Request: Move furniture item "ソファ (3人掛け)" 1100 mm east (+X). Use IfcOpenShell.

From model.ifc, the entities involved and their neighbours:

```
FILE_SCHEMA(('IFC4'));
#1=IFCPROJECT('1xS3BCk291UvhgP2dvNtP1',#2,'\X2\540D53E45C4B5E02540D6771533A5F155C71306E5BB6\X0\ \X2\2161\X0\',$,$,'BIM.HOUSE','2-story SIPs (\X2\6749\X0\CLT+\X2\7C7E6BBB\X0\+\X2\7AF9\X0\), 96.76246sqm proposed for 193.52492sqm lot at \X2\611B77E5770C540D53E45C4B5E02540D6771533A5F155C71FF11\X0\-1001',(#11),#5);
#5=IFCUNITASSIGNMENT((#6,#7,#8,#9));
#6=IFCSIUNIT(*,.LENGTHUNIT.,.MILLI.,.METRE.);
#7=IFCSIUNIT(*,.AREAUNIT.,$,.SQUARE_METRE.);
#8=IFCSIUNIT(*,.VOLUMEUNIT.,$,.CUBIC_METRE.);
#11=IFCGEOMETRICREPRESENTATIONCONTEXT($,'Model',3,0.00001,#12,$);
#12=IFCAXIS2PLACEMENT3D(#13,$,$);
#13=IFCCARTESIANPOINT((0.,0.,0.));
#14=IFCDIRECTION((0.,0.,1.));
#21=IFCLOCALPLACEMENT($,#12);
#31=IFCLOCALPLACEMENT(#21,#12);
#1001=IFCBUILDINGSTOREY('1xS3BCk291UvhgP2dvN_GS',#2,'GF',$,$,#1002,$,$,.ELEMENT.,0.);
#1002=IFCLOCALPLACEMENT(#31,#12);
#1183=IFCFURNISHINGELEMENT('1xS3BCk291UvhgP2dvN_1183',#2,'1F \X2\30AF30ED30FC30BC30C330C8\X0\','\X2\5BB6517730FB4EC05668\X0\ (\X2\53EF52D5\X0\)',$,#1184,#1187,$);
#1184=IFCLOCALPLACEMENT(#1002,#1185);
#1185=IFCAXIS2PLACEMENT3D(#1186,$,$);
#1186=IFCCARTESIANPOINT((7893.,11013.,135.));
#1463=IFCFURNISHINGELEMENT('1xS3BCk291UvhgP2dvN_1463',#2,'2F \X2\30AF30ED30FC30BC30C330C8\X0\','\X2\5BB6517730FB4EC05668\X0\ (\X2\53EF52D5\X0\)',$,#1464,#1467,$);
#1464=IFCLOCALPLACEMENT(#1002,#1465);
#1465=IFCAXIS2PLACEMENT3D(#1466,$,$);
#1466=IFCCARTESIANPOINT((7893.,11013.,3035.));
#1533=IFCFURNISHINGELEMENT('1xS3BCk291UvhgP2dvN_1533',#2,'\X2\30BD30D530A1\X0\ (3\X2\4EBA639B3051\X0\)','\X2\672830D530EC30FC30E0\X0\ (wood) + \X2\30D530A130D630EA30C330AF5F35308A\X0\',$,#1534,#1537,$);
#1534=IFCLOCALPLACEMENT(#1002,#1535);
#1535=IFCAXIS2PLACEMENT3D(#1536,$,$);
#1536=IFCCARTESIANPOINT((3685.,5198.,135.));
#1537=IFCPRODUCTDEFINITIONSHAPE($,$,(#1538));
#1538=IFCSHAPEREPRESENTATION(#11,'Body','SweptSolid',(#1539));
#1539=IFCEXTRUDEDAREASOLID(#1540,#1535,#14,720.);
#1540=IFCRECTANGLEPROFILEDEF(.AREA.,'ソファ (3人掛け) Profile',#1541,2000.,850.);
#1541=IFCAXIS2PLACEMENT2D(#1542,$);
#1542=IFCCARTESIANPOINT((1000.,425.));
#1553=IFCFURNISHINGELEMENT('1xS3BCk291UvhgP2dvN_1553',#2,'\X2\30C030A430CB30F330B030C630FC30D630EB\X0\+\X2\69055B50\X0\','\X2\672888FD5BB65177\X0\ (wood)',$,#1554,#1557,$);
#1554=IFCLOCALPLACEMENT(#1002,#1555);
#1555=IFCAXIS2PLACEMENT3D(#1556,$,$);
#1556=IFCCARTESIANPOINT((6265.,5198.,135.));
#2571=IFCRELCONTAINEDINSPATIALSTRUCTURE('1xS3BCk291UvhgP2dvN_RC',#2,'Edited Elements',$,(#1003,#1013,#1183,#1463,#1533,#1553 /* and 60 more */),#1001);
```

```python
import ifcopenshell
import ifcopenshell.api.geometry
import ifcopenshell.util.placement
import ifcopenshell.util.unit

model = ifcopenshell.open("model.ifc")
unit_scale = ifcopenshell.util.unit.calculate_unit_scale(model)

item = model.by_guid("1xS3BCk291UvhgP2dvN_1533")
matrix = ifcopenshell.util.placement.get_local_placement(item.ObjectPlacement)
matrix[0, 3] += 1.1 / unit_scale
ifcopenshell.api.geometry.edit_object_placement(model, product=item, matrix=matrix, is_si=False)

print(ifcopenshell.util.placement.get_local_placement(item.ObjectPlacement).round(3) + 0.0)

model.write("model-out.ifc")
```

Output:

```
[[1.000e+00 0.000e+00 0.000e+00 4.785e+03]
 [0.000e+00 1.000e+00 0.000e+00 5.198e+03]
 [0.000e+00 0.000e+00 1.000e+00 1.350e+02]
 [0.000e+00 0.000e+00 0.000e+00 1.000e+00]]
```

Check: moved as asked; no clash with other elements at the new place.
